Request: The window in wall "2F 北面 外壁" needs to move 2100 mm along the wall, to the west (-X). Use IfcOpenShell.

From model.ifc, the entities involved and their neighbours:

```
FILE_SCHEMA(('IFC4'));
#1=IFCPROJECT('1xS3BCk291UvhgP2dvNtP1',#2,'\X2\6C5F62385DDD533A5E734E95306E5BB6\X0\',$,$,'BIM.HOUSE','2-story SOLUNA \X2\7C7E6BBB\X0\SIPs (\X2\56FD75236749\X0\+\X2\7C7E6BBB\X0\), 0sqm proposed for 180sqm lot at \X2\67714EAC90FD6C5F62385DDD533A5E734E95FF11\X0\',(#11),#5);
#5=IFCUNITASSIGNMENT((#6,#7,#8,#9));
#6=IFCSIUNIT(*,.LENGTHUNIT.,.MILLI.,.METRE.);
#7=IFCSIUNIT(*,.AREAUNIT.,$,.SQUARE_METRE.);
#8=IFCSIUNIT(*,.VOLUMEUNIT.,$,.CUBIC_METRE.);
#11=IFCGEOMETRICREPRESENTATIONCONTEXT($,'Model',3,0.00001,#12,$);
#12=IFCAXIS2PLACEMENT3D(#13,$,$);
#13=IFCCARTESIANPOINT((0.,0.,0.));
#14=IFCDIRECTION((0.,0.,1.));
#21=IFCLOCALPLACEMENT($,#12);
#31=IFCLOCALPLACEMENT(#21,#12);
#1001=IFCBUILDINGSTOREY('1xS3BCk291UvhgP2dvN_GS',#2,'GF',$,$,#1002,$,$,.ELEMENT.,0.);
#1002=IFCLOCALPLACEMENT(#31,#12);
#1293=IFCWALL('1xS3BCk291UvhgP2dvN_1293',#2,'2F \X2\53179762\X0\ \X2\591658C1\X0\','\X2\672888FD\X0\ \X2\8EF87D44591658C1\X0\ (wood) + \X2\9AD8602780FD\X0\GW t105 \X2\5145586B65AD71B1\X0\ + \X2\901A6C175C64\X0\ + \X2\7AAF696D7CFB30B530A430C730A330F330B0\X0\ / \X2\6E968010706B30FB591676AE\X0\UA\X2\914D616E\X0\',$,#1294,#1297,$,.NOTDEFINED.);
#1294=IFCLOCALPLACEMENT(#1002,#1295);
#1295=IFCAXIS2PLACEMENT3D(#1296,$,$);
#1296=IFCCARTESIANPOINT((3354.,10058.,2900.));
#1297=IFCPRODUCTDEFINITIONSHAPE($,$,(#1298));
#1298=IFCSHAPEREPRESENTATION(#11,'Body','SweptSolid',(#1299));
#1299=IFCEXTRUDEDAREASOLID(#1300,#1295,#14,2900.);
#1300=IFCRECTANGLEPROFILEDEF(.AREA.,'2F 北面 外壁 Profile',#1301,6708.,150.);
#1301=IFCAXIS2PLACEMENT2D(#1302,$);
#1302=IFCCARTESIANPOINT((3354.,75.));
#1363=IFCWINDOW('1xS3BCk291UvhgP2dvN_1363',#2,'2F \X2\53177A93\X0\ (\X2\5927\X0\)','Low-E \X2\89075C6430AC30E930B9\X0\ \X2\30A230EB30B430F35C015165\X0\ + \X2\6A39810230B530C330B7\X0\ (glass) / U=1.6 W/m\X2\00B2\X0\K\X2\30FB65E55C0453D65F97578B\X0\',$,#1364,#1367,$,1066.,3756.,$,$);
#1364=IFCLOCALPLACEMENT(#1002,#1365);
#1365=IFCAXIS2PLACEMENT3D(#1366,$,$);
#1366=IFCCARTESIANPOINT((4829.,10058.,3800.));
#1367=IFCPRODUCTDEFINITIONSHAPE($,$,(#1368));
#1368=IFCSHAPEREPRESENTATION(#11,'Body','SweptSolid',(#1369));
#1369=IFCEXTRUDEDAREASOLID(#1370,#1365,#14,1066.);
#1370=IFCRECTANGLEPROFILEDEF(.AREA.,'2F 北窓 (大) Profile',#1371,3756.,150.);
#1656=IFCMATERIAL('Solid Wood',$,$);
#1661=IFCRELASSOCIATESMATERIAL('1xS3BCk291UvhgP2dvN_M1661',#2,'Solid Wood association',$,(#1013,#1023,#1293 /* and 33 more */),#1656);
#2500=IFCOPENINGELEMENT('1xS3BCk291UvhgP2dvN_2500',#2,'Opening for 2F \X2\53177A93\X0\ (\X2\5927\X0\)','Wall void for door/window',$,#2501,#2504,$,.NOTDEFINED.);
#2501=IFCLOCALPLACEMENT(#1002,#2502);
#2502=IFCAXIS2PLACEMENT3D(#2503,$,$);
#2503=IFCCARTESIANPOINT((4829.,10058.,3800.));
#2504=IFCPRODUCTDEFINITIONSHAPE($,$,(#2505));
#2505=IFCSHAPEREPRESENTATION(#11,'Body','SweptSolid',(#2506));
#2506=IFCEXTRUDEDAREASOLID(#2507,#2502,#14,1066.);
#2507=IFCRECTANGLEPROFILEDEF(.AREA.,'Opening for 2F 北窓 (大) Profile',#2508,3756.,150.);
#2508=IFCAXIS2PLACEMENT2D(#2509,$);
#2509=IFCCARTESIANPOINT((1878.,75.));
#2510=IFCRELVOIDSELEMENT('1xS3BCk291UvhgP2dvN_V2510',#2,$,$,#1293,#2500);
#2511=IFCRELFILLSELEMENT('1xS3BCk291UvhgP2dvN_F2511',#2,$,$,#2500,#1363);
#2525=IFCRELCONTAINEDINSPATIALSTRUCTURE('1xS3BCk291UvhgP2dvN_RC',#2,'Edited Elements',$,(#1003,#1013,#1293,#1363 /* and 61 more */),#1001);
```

```python
import ifcopenshell
import ifcopenshell.api.geometry
import ifcopenshell.util.placement

model = ifcopenshell.open("model.ifc")

window = model.by_guid("1xS3BCk291UvhgP2dvN_1363")
opening = window.FillsVoids[0].RelatingOpeningElement
wall = opening.VoidsElements[0].RelatingBuildingElement

wall_matrix = ifcopenshell.util.placement.get_local_placement(wall.ObjectPlacement)
shift = wall_matrix[:3, 0] * -2100.0
before = ifcopenshell.util.placement.get_local_placement(window.ObjectPlacement)[:3, 3].copy()

# The window is not placed relative to its opening, so move both.
for product in (opening, window):
    matrix = ifcopenshell.util.placement.get_local_placement(product.ObjectPlacement)
    matrix[:3, 3] += shift
    ifcopenshell.api.geometry.edit_object_placement(model, product=product, matrix=matrix, is_si=False)

after = ifcopenshell.util.placement.get_local_placement(window.ObjectPlacement)[:3, 3]
print("window moved by", (after - before).round(3) + 0.0)

model.write("model_rev.ifc")
```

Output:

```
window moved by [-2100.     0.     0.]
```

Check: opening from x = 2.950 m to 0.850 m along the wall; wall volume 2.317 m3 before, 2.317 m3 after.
